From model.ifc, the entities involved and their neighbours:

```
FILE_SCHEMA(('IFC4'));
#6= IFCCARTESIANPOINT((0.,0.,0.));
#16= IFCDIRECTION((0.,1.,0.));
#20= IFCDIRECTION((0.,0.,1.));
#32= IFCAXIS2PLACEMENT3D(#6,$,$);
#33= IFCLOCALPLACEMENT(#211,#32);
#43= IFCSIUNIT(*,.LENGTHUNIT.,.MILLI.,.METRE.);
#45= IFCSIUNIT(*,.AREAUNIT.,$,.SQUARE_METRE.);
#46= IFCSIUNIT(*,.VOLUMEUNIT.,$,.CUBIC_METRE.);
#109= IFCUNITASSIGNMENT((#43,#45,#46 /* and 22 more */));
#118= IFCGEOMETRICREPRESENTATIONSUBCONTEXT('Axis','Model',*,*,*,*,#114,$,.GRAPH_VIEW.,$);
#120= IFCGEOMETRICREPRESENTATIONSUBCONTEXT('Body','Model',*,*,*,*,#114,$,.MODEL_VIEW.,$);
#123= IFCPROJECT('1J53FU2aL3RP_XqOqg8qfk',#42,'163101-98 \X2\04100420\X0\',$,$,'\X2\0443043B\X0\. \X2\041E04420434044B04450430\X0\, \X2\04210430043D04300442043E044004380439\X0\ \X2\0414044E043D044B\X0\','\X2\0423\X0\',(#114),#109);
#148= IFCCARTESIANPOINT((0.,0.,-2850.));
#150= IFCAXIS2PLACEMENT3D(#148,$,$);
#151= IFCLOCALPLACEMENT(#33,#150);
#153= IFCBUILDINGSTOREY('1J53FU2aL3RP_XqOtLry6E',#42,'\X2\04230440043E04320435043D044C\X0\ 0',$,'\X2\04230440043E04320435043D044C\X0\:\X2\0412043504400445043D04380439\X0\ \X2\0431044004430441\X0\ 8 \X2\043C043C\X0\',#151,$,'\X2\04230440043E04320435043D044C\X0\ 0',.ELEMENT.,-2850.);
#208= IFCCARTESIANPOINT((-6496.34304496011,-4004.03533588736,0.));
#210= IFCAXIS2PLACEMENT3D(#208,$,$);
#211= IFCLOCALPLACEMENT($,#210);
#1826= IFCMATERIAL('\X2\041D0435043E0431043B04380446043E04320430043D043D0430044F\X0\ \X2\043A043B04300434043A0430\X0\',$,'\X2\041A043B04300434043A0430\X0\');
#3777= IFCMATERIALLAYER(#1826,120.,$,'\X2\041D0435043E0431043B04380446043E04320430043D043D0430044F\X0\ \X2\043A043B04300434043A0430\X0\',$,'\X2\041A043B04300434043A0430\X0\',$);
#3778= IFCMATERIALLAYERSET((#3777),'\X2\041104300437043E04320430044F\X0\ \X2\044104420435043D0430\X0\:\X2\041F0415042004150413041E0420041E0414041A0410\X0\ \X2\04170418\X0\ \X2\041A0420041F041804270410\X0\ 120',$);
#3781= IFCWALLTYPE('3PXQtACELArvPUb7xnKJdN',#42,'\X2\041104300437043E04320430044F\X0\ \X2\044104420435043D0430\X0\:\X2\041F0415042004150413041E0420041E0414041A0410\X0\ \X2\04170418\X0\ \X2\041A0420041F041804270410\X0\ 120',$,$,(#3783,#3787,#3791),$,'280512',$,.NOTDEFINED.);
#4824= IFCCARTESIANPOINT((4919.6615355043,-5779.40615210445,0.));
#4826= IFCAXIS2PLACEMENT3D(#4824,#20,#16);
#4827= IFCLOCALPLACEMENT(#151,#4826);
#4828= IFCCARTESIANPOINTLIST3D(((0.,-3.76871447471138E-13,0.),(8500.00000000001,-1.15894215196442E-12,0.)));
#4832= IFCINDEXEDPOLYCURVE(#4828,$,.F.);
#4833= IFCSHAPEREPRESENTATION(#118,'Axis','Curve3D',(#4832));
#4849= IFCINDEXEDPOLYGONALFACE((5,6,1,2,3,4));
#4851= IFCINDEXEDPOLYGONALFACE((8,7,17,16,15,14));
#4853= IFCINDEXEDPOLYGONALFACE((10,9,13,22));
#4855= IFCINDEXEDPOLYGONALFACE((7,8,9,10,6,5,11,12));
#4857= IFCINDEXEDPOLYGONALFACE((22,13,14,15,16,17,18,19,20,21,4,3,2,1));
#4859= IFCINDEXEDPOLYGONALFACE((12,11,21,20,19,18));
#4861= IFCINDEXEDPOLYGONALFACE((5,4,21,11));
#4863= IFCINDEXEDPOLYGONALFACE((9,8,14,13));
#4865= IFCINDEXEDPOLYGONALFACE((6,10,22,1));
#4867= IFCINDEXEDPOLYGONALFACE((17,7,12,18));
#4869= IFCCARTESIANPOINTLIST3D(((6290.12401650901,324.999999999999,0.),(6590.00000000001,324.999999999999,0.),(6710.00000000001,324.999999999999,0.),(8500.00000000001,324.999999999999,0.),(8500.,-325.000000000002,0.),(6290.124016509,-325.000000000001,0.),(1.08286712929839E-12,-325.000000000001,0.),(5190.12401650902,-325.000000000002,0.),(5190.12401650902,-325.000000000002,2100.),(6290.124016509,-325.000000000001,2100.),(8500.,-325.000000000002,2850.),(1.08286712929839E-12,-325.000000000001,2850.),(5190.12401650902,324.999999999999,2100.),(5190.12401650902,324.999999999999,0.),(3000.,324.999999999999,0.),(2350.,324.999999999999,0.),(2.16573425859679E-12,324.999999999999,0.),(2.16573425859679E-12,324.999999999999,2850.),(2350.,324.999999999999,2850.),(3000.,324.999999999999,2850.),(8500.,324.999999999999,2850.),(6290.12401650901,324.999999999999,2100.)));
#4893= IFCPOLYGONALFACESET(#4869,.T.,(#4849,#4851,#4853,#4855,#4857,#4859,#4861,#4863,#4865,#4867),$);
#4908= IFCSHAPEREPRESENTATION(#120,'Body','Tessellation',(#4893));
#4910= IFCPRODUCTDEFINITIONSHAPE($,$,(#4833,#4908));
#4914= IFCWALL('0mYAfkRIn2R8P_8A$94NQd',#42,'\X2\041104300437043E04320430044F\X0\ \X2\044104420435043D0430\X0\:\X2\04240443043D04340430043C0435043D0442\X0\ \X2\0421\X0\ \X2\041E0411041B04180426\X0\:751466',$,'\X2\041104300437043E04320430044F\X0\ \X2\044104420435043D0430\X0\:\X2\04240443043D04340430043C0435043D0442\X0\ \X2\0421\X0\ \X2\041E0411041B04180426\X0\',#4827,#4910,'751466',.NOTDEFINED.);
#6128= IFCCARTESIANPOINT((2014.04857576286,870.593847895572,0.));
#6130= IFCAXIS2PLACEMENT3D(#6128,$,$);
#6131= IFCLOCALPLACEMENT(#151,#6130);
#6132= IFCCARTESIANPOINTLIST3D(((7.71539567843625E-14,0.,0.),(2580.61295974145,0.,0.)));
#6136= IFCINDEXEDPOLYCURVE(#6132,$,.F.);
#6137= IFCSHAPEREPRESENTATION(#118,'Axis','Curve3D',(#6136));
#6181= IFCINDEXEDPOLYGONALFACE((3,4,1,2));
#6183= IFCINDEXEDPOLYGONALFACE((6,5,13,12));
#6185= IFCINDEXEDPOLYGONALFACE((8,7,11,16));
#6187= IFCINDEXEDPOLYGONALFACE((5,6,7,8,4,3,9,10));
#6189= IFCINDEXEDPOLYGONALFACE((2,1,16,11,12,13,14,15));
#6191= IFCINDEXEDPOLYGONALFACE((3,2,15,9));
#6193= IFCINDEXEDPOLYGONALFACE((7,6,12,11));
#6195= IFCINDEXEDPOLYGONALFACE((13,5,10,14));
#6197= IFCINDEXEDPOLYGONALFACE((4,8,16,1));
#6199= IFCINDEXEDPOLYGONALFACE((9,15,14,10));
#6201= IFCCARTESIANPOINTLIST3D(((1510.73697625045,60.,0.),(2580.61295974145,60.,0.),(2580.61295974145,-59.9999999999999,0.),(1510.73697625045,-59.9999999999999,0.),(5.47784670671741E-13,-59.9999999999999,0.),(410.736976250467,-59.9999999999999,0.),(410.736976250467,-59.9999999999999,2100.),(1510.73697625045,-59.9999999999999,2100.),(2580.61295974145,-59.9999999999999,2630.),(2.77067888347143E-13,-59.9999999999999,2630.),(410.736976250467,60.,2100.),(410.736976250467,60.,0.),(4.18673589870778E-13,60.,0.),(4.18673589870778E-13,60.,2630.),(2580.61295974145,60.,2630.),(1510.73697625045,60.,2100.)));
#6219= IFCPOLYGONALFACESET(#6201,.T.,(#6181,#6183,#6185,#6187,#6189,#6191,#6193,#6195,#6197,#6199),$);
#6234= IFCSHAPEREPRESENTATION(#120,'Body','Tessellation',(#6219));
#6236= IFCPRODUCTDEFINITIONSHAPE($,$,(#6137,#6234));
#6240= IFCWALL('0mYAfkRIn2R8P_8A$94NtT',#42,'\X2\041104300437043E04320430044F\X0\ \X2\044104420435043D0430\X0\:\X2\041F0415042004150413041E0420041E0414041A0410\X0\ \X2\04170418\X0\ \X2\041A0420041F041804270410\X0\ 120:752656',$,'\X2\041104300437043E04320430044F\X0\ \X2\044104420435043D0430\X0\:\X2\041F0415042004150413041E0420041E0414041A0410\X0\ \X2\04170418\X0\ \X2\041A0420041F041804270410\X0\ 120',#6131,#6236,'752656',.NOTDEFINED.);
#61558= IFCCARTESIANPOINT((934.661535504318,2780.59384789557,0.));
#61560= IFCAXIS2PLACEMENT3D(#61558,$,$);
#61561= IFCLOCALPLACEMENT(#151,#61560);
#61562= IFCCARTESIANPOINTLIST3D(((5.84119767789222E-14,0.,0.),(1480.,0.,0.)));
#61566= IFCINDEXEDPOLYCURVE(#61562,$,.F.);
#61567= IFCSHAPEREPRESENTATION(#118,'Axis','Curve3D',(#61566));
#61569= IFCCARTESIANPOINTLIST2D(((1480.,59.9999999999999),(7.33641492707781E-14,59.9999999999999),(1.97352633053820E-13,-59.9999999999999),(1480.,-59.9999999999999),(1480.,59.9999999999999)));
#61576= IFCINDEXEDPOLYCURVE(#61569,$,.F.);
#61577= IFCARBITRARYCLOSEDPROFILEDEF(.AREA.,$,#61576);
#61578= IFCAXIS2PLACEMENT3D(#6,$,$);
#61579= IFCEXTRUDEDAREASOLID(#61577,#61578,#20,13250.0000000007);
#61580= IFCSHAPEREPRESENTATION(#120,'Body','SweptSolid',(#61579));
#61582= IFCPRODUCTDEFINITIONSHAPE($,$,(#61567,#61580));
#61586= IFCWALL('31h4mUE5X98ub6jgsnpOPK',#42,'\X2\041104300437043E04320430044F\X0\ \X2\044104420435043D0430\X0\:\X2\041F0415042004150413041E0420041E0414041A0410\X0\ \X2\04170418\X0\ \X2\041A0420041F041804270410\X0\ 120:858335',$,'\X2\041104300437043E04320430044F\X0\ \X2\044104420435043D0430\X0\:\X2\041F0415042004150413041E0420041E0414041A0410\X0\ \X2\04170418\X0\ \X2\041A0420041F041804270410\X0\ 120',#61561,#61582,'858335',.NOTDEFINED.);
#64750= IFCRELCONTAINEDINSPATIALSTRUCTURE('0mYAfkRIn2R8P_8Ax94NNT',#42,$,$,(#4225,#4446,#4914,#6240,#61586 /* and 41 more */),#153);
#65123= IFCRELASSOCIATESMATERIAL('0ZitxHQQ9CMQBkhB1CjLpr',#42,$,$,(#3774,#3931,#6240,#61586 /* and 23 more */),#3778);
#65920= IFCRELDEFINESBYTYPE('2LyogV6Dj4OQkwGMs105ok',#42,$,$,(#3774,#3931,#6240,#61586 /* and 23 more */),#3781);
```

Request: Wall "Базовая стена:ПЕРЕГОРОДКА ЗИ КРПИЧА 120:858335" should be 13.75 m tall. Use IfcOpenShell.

```python
import ifcopenshell
import ifcopenshell.geom
import ifcopenshell.util.representation
import ifcopenshell.util.shape
import ifcopenshell.util.unit

model = ifcopenshell.open("model.ifc")
unit_scale = ifcopenshell.util.unit.calculate_unit_scale(model)
settings = ifcopenshell.geom.settings()


def volume(element):
    """Net volume in cubic metres, openings subtracted."""
    shape = ifcopenshell.geom.create_shape(settings, element)
    return ifcopenshell.util.shape.get_volume(shape.geometry)


wall = model.by_id(61586)
before = volume(wall)

body = ifcopenshell.util.representation.get_representation(wall, "Model", "Body")
solid = body.Items[0]
old_height = solid.Depth
solid.Depth = 13.75 / unit_scale
after = volume(wall)

print(f"height {old_height:g} -> {solid.Depth:g}, volume {before:.3f} -> {after:.3f} m3")

model.write("model_updated.ifc")
```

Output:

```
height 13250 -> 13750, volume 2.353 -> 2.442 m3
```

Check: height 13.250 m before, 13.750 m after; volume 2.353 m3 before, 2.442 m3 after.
